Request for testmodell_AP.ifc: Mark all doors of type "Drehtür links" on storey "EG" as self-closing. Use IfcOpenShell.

First a look at what the model holds.

```python
import ifcopenshell
import ifcopenshell.util.element

model = ifcopenshell.open("testmodell_AP.ifc")
print(model.schema)
storey = next(s for s in model.by_type("IfcBuildingStorey") if s.Name == "EG")
doors = [e for e in ifcopenshell.util.element.get_decomposition(storey) if e.is_a("IfcDoor")]
seen = {}
for e in doors:
    element_type = ifcopenshell.util.element.get_type(e)
    key = (element_type.Name if element_type != e and element_type else None, ifcopenshell.util.element.get_pset(e, "Pset_DoorCommon", "SelfClosing"))
    seen[key] = seen.get(key, 0) + 1
for (name, value), count in sorted(seen.items(), key=str):
    print(count, "x", name, "|", value)
```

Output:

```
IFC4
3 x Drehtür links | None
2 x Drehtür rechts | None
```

```python
import ifcopenshell
import ifcopenshell.api.pset
import ifcopenshell.util.element

model = ifcopenshell.open("testmodell_AP.ifc")

storey = next(s for s in model.by_type("IfcBuildingStorey") if s.Name == "EG")
doors = [e for e in ifcopenshell.util.element.get_decomposition(storey) if e.is_a("IfcDoor")]

count = 0
for e in doors:
    element_type = ifcopenshell.util.element.get_type(e)
    if element_type in (None, e) or element_type.Name != "Drehtür links":
        continue
    # add_pset returns the element's existing set when there is one.
    pset = ifcopenshell.api.pset.add_pset(model, product=e, name="Pset_DoorCommon")
    ifcopenshell.api.pset.edit_pset(model, pset=pset, properties={"SelfClosing": True})
    count += 1

print(count, "doors updated")

model.write("testmodell_AP_rev.ifc")
```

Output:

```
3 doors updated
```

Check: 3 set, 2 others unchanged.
